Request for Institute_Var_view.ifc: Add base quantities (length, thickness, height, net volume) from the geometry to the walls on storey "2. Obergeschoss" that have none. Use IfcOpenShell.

First a look at what the model holds.

```python
import ifcopenshell
import ifcopenshell.util.element
import ifcopenshell.util.unit

model = ifcopenshell.open("Institute_Var_view.ifc")
print(model.schema)
for unit_type in ("LENGTHUNIT", "AREAUNIT", "VOLUMEUNIT"):
    print(unit_type, ifcopenshell.util.unit.calculate_unit_scale(model, unit_type))
storey = next(s for s in model.by_type("IfcBuildingStorey") if s.Name == "2. Obergeschoss")
walls = [e for e in ifcopenshell.util.element.get_decomposition(storey) if e.is_a("IfcWall")]
for e in sorted(walls, key=lambda e: e.id()):
    print(e.id(), e.is_a(), e.Name, list(ifcopenshell.util.element.get_psets(e, qtos_only=True)), sep=" | ")
```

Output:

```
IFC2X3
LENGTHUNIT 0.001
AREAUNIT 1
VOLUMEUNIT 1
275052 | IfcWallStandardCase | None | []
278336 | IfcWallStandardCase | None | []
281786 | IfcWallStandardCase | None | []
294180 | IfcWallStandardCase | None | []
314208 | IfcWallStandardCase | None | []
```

```python
import ifcopenshell
import ifcopenshell.api.pset
import ifcopenshell.geom
import ifcopenshell.util.element
import ifcopenshell.util.shape
import ifcopenshell.util.unit

model = ifcopenshell.open("Institute_Var_view.ifc")
unit_scale = ifcopenshell.util.unit.calculate_unit_scale(model)
volume_scale = ifcopenshell.util.unit.calculate_unit_scale(model, "VOLUMEUNIT")
settings = ifcopenshell.geom.settings()

storey = next(s for s in model.by_type("IfcBuildingStorey") if s.Name == "2. Obergeschoss")
walls = [e for e in ifcopenshell.util.element.get_decomposition(storey) if e.is_a("IfcWall")]

for e in sorted(walls, key=lambda e: e.id()):
    if ifcopenshell.util.element.get_psets(e, qtos_only=True, should_inherit=False):
        continue
    # Geometry comes back in metres, in the element's own axes.
    shape = ifcopenshell.geom.create_shape(settings, e)
    values = {
        "Length": ifcopenshell.util.shape.get_x(shape.geometry) / unit_scale,
        "Width": ifcopenshell.util.shape.get_y(shape.geometry) / unit_scale,
        "Height": ifcopenshell.util.shape.get_z(shape.geometry) / unit_scale,
        "NetVolume": ifcopenshell.util.shape.get_volume(shape.geometry) / volume_scale,
    }
    qto = ifcopenshell.api.pset.add_qto(model, product=e, name="BaseQuantities")
    ifcopenshell.api.pset.edit_qto(model, qto=qto, properties=values)
    print(e.id(), {k: round(v, 3) for k, v in values.items()})

model.write("Institute_Var_view_rev.ifc")
```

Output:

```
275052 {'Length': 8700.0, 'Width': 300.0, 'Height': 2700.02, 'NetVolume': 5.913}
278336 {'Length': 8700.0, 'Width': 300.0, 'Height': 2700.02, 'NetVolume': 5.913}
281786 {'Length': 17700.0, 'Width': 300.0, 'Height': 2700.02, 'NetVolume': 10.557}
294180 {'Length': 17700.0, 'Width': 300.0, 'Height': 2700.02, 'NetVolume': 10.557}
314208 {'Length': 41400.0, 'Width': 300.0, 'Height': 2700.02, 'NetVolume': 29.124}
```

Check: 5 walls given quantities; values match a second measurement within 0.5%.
